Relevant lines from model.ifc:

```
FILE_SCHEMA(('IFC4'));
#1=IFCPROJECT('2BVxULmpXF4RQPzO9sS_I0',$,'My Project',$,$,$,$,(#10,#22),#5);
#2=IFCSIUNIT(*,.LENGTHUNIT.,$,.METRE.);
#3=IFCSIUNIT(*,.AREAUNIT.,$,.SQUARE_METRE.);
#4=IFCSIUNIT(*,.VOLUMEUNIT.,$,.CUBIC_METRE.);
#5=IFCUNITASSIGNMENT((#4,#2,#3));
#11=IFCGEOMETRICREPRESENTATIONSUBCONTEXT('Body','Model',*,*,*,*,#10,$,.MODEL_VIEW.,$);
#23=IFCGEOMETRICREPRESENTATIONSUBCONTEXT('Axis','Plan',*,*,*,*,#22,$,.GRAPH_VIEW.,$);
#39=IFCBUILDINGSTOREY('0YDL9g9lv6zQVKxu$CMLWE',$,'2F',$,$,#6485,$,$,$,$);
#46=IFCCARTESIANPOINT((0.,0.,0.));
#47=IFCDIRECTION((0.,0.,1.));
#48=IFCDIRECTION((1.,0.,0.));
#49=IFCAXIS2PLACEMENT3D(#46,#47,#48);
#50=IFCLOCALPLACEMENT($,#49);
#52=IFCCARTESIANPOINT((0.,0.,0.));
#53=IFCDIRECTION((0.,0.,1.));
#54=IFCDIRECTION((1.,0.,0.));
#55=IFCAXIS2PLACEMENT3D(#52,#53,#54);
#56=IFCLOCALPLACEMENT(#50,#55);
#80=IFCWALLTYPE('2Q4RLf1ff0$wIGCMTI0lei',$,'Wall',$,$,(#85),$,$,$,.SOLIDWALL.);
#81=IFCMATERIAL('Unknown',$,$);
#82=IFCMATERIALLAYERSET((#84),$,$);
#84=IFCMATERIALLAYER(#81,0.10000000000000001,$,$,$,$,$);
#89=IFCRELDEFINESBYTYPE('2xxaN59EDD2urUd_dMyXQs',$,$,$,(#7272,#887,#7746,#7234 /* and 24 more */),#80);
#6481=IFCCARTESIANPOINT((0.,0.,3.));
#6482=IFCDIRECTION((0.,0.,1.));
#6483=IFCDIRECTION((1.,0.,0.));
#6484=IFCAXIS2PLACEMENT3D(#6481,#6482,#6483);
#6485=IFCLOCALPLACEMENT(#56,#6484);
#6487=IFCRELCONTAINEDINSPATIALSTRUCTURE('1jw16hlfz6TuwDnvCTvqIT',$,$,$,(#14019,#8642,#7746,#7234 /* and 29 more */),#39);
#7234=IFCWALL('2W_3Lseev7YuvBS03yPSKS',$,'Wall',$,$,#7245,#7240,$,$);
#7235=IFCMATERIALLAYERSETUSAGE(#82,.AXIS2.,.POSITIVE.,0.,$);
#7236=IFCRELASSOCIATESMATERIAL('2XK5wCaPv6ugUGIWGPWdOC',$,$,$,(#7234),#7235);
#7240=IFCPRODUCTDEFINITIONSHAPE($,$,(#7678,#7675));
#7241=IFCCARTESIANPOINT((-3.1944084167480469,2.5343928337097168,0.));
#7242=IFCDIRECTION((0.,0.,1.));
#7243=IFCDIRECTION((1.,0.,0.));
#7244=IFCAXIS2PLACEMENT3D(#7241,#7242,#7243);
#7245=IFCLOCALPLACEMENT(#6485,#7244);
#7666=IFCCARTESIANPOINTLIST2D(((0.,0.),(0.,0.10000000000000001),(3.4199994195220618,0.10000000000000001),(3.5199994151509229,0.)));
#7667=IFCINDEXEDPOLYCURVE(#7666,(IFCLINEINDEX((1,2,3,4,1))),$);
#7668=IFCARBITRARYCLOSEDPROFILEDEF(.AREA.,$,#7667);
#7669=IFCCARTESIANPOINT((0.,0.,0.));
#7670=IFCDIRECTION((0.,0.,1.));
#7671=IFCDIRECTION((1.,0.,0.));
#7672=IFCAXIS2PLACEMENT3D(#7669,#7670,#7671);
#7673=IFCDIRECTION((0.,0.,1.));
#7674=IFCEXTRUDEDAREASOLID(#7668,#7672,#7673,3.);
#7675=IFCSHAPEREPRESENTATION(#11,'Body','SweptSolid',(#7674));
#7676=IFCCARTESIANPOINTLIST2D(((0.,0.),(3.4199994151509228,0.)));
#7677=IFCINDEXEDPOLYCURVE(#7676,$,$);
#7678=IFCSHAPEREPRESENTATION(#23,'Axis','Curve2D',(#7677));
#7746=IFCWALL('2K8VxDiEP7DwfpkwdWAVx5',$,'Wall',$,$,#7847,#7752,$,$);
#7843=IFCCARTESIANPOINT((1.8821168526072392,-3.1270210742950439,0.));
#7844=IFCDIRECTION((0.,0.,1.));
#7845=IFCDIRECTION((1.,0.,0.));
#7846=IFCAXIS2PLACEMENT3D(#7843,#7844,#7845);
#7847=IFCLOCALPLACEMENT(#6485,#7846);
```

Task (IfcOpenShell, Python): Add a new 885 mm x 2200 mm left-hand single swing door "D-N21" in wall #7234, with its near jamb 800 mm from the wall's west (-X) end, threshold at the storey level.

```python
import numpy as np
import ifcopenshell
import ifcopenshell.api.feature
import ifcopenshell.api.geometry
import ifcopenshell.api.root
import ifcopenshell.api.spatial
import ifcopenshell.geom
import ifcopenshell.util.element
import ifcopenshell.util.placement
import ifcopenshell.util.representation
import ifcopenshell.util.shape
import ifcopenshell.util.unit

model = ifcopenshell.open("model.ifc")
unit_scale = ifcopenshell.util.unit.calculate_unit_scale(model)
settings = ifcopenshell.geom.settings()


def volume(element):
    """Net volume in cubic metres, openings subtracted."""
    shape = ifcopenshell.geom.create_shape(settings, element)
    return ifcopenshell.util.shape.get_volume(shape.geometry)


wall = model.by_id(7234)
storey = ifcopenshell.util.element.get_container(wall, ifc_class="IfcBuildingStorey")
context = ifcopenshell.util.representation.get_context(model, "Model", "Body", "MODEL_VIEW")
before = volume(wall)

width, height, from_end, sill = 0.885, 2.2, 0.8, 0.0  # metres

# The wall runs along its own X axis, and the end named is its -X end.
wall_shape = ifcopenshell.geom.create_shape(settings, wall)
x, y, z = ifcopenshell.util.shape.get_vertices(wall_shape.geometry).T
start = x.min() + from_end
face, thickness = float(y.min()), float(y.max() - y.min())
wall_matrix = ifcopenshell.util.placement.get_local_placement(wall.ObjectPlacement)
level = ifcopenshell.util.placement.get_local_placement(storey.ObjectPlacement)[2, 3]


def in_wall(x, y):
    """Placement at x, y metres in the wall's axes, at sill height."""
    matrix = wall_matrix.copy()
    matrix[:, 3] = wall_matrix @ np.array([x / unit_scale, y / unit_scale, 0.0, 1.0])
    matrix[2, 3] = level + sill / unit_scale
    return matrix


# Opening: a box that overshoots both wall faces by 50 mm.
opening = ifcopenshell.api.root.create_entity(model, ifc_class="IfcOpeningElement", predefined_type="OPENING")
box = ifcopenshell.api.geometry.add_wall_representation(
    model, context=context, length=width, height=height, thickness=thickness + 0.1
)
ifcopenshell.api.geometry.assign_representation(model, product=opening, representation=box)
ifcopenshell.api.geometry.edit_object_placement(model, product=opening, matrix=in_wall(start, face - 0.05), is_si=False)
ifcopenshell.api.feature.add_feature(model, feature=opening, element=wall)

door = ifcopenshell.api.root.create_entity(model, ifc_class="IfcDoor", name="D-N21", predefined_type="DOOR")
door.OverallWidth, door.OverallHeight = width / unit_scale, height / unit_scale
door.OperationType = "SINGLE_SWING_LEFT"
body = ifcopenshell.api.geometry.add_door_representation(
    model,
    context=context,
    overall_width=door.OverallWidth,
    overall_height=door.OverallHeight,
    operation_type="SINGLE_SWING_LEFT",
    lining_properties={"LiningDepth": thickness / unit_scale, "ThresholdDepth": thickness / unit_scale},
)
ifcopenshell.api.geometry.assign_representation(model, product=door, representation=body)
ifcopenshell.api.spatial.assign_container(model, products=[door], relating_structure=storey)
ifcopenshell.api.feature.add_filling(model, opening=opening, element=door)

# The lining spans the wall, so the door starts at the wall face.
ifcopenshell.api.geometry.edit_object_placement(model, product=door, matrix=in_wall(start, face), is_si=False)

after = volume(wall)

print(f"wall volume {before:.3f} -> {after:.3f} m3")

model.write("model_v2.ifc")
```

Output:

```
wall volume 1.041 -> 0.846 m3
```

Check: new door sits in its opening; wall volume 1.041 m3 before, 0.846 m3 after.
